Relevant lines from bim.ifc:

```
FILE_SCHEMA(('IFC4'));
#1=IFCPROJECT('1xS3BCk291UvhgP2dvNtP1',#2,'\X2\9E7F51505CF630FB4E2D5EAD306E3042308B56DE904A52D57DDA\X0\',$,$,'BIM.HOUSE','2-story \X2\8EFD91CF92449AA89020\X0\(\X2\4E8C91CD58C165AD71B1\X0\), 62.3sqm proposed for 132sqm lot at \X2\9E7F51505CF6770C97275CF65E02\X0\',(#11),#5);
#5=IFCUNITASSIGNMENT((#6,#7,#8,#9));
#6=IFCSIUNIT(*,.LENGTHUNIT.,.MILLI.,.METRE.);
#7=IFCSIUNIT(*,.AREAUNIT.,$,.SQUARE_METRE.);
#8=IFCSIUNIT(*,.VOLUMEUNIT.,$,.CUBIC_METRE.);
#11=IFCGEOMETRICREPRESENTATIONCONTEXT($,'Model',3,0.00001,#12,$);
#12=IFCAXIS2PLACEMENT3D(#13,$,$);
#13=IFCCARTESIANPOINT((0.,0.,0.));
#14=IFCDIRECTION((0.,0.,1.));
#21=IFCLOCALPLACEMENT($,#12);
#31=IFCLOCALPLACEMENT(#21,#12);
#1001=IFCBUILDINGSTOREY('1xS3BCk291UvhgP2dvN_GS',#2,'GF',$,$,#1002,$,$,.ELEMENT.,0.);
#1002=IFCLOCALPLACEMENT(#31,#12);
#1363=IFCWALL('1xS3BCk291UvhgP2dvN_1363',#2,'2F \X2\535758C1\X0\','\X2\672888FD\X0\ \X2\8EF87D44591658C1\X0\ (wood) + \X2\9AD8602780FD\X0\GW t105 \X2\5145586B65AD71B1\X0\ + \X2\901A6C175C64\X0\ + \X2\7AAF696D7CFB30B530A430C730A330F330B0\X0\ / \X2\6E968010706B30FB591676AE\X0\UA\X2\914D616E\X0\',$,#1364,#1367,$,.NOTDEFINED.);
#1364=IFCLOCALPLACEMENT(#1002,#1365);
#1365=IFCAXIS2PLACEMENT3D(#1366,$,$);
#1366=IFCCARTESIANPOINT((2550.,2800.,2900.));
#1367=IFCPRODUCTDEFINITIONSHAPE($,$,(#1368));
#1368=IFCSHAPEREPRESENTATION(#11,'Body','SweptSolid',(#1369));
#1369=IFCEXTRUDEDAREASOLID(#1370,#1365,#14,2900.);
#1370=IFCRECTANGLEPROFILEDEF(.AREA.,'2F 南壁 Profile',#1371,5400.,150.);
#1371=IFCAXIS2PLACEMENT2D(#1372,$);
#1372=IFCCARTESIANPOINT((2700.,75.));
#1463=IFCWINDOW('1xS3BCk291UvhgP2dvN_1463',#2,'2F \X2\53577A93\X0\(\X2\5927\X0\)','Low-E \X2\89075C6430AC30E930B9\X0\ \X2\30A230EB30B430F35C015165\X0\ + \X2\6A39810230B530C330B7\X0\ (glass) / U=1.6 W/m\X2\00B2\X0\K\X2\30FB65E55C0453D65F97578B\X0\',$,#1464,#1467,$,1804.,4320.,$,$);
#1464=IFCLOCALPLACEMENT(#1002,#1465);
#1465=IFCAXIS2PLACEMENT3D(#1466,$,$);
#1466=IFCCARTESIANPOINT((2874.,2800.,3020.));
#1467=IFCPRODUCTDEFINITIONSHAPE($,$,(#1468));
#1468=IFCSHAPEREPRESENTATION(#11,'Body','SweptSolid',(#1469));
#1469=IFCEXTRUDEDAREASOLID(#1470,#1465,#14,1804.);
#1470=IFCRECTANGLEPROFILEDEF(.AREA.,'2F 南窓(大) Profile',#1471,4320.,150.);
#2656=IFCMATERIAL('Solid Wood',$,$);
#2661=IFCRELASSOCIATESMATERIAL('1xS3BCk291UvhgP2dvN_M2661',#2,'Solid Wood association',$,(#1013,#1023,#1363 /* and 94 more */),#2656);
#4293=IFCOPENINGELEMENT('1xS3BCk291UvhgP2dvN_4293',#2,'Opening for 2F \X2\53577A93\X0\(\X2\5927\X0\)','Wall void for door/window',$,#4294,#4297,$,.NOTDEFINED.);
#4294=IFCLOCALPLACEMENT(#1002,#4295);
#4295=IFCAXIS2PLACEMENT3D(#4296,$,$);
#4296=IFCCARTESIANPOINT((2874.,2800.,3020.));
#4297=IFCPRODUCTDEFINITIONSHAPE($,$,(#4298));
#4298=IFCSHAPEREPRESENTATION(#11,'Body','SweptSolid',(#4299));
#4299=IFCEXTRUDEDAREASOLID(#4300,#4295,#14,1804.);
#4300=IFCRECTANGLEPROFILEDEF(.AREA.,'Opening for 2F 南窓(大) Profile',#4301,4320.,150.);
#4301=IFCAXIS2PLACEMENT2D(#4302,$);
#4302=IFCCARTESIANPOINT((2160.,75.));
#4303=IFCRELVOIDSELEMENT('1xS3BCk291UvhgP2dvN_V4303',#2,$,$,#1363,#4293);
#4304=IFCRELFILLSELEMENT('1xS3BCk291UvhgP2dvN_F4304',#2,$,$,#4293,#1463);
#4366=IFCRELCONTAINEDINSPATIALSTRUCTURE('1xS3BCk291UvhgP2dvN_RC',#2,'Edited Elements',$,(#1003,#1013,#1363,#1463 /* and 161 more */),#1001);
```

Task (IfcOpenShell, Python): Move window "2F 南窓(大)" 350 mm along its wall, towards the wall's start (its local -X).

```python
import ifcopenshell
import ifcopenshell.api.geometry
import ifcopenshell.util.placement

model = ifcopenshell.open("bim.ifc")

window = model.by_guid("1xS3BCk291UvhgP2dvN_1463")
opening = window.FillsVoids[0].RelatingOpeningElement
wall = opening.VoidsElements[0].RelatingBuildingElement

wall_matrix = ifcopenshell.util.placement.get_local_placement(wall.ObjectPlacement)
shift = wall_matrix[:3, 0] * -350.0
before = ifcopenshell.util.placement.get_local_placement(window.ObjectPlacement)[:3, 3].copy()

# The window is not placed relative to its opening, so move both.
for product in (opening, window):
    matrix = ifcopenshell.util.placement.get_local_placement(product.ObjectPlacement)
    matrix[:3, 3] += shift
    ifcopenshell.api.geometry.edit_object_placement(model, product=product, matrix=matrix, is_si=False)

after = ifcopenshell.util.placement.get_local_placement(window.ObjectPlacement)[:3, 3]
print("window moved by", (after - before).round(3) + 0.0)

model.write("bim-out.ifc")
```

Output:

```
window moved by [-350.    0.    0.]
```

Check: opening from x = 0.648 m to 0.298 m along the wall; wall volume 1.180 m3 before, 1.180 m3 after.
